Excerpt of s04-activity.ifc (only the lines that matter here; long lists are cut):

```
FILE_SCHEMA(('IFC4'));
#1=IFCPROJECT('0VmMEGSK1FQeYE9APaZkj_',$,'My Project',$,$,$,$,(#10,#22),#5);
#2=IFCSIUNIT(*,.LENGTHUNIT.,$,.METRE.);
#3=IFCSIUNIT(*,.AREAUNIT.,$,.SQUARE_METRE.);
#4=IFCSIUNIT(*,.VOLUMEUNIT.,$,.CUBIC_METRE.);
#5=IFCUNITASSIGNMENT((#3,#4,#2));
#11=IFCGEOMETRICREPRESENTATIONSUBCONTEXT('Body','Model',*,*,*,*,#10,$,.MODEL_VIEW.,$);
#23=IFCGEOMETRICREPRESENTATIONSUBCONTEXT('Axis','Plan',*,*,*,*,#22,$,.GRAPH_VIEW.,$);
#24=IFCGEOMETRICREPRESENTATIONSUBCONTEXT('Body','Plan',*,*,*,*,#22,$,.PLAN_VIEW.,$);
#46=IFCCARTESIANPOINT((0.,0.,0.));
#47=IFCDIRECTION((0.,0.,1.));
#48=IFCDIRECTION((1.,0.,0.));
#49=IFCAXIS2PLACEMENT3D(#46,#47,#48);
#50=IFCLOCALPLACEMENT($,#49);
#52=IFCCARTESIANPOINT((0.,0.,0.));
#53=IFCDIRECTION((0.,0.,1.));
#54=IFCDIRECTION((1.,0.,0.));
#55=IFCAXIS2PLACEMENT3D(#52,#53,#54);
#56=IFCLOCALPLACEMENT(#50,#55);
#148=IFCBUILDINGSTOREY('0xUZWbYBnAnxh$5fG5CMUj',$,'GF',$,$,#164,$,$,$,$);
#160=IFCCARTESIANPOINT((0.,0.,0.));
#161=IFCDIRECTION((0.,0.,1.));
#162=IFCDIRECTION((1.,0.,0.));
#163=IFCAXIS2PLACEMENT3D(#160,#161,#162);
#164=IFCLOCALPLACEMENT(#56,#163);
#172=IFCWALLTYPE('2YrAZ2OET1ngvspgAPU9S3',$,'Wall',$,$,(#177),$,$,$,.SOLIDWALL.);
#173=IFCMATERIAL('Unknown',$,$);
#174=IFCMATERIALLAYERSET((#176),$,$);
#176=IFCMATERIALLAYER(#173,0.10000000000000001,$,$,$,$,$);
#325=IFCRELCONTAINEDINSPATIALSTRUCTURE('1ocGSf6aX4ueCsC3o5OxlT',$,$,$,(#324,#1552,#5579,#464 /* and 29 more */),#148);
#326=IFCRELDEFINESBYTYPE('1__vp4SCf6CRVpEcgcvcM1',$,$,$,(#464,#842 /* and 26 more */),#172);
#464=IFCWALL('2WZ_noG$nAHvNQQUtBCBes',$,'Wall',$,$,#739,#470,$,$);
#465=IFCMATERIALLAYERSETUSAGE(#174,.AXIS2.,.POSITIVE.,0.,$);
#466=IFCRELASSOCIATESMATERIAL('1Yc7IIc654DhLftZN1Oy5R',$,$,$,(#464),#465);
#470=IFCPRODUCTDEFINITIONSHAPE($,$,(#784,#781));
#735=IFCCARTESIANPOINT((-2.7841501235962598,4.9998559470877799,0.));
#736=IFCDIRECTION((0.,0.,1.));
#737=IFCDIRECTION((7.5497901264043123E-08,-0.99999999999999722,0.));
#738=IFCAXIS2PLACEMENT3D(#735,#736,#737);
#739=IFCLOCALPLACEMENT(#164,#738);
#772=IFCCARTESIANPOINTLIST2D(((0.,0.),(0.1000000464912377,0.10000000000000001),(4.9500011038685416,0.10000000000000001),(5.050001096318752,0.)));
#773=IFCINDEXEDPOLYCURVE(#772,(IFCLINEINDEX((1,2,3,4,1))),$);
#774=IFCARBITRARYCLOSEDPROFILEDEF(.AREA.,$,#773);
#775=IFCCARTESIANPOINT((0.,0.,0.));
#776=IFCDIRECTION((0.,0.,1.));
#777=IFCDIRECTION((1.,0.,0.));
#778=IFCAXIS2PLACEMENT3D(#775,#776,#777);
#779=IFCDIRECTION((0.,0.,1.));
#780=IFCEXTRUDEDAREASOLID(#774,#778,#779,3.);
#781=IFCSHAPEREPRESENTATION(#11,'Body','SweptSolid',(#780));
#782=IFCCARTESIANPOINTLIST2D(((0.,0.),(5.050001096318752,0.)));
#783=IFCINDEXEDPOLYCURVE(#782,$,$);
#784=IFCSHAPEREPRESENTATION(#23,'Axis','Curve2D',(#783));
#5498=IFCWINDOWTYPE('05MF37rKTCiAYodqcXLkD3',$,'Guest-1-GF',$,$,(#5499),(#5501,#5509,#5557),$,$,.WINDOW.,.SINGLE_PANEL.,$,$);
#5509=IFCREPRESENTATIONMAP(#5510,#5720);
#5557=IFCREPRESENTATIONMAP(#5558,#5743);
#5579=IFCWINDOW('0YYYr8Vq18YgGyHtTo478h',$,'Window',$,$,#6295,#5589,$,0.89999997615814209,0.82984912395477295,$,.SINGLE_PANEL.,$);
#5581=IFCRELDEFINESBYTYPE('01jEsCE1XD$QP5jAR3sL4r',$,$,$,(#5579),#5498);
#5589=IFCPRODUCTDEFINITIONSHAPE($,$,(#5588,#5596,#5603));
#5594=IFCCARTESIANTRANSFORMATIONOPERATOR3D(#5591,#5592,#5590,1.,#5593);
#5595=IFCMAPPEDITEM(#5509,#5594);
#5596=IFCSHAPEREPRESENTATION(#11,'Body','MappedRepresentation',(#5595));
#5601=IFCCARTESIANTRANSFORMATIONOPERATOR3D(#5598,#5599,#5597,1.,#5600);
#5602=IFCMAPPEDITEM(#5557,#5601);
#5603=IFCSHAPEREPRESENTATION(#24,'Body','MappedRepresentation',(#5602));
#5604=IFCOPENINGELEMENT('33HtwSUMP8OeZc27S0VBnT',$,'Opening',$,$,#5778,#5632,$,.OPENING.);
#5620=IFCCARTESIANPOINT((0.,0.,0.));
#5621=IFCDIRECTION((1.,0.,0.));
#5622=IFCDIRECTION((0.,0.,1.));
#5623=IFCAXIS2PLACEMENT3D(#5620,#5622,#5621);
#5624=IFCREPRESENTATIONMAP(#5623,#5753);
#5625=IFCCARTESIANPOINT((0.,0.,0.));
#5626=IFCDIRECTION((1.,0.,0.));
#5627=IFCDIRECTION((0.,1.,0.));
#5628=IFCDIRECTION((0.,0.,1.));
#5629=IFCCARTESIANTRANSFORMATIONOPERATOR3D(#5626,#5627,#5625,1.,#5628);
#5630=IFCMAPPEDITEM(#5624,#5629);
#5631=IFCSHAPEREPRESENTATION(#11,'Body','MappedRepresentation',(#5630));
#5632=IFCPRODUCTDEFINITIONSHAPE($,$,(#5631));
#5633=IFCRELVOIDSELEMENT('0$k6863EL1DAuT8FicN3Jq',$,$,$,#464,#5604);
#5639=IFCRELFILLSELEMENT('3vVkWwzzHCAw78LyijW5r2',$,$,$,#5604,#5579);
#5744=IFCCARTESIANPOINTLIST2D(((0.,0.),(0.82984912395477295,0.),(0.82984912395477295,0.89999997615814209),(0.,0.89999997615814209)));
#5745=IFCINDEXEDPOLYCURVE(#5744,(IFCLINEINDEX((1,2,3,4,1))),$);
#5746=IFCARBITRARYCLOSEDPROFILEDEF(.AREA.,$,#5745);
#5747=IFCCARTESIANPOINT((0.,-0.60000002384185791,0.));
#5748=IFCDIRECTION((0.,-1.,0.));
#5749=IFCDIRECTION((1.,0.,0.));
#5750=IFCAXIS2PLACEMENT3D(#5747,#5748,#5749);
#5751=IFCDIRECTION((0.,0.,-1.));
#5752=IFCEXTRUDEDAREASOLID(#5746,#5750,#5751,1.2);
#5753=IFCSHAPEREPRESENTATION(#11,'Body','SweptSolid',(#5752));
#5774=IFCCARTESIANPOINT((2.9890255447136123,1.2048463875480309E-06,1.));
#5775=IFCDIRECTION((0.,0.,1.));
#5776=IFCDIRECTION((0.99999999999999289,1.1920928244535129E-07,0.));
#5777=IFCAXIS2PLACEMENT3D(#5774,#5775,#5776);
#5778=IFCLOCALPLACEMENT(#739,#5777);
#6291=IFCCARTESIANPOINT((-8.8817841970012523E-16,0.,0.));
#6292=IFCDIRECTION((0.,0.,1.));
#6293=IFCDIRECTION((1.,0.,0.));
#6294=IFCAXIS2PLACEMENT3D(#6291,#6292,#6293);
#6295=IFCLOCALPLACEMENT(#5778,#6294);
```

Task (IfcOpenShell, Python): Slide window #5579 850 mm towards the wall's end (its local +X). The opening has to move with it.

```python
import ifcopenshell
import ifcopenshell.api.geometry
import ifcopenshell.util.placement

model = ifcopenshell.open("s04-activity.ifc")

window = model.by_guid("0YYYr8Vq18YgGyHtTo478h")
opening = window.FillsVoids[0].RelatingOpeningElement
wall = opening.VoidsElements[0].RelatingBuildingElement

wall_matrix = ifcopenshell.util.placement.get_local_placement(wall.ObjectPlacement)
shift = wall_matrix[:3, 0] * 0.85
before = ifcopenshell.util.placement.get_local_placement(window.ObjectPlacement)[:3, 3].copy()

# The window is placed relative to its opening, so it follows when the opening moves.
matrix = ifcopenshell.util.placement.get_local_placement(opening.ObjectPlacement)
matrix[:3, 3] += shift
ifcopenshell.api.geometry.edit_object_placement(
    model, product=opening, matrix=matrix, is_si=False, should_transform_children=True
)

after = ifcopenshell.util.placement.get_local_placement(window.ObjectPlacement)[:3, 3]
print("window moved by", (after - before).round(3) + 0.0)

model.write("s04-activity_rev.ifc")
```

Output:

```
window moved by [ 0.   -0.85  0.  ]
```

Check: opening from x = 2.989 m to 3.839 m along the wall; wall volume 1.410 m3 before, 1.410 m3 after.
